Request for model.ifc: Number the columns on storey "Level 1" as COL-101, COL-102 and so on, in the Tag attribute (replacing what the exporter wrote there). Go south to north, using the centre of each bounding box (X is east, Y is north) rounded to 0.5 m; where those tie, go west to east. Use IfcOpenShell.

First a look at what the model holds.

```python
import ifcopenshell
import ifcopenshell.util.element
import ifcopenshell.util.placement

model = ifcopenshell.open("model.ifc")
print(model.schema)
storey = next(s for s in model.by_type("IfcBuildingStorey") if s.Name == "Level 1")
columns = [e for e in ifcopenshell.util.element.get_decomposition(storey) if e.is_a("IfcColumn")]
for e in sorted(columns, key=lambda e: e.id()):
    origin = ifcopenshell.util.placement.get_local_placement(e.ObjectPlacement)[:3, 3]
    print(e.id(), e.Tag, e.Name, origin.round(2) + 0.0, sep=" | ")
```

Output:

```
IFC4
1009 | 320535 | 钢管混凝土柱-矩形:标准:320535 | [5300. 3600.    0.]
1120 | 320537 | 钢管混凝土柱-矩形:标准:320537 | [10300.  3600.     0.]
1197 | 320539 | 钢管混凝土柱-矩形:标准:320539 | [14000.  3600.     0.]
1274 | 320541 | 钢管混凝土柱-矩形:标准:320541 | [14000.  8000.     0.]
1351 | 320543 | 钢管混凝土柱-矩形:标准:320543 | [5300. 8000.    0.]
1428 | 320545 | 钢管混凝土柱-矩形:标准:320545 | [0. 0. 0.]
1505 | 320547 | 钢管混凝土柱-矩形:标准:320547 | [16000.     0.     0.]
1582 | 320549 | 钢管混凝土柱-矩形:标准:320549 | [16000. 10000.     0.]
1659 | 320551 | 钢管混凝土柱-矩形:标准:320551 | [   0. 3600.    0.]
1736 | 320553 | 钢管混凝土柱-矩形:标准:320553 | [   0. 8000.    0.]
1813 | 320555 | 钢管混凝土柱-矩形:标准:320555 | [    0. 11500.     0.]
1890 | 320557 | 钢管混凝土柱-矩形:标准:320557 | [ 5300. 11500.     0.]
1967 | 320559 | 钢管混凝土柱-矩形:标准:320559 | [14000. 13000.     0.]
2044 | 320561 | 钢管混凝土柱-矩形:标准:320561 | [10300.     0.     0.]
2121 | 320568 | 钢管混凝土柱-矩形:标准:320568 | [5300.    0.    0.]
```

```python
import ifcopenshell
import ifcopenshell.geom
import ifcopenshell.util.element
import ifcopenshell.util.shape

model = ifcopenshell.open("model.ifc")
settings = ifcopenshell.geom.settings()
settings.set("use-world-coords", True)


def centre(element):
    shape = ifcopenshell.geom.create_shape(settings, element)
    return ifcopenshell.util.shape.get_bbox_centroid(shape.geometry)


storey = next(s for s in model.by_type("IfcBuildingStorey") if s.Name == "Level 1")
columns = [e for e in ifcopenshell.util.element.get_decomposition(storey) if e.is_a("IfcColumn")]

# Insertion points can sit at a corner or the storey origin, so sort by the geometry (in metres).
centres = {e: centre(e) for e in columns}
columns.sort(key=lambda e: (round(centres[e][1] / 0.5), centres[e][0]))

for i, e in enumerate(columns, start=1):
    number = f"COL-1{i:02d}"
    e.Tag = number
    print(e.id(), number)

model.write("model_edited.ifc")
```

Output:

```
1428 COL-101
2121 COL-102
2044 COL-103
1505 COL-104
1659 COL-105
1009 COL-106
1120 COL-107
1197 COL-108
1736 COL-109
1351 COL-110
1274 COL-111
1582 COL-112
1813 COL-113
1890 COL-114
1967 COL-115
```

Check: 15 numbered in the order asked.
